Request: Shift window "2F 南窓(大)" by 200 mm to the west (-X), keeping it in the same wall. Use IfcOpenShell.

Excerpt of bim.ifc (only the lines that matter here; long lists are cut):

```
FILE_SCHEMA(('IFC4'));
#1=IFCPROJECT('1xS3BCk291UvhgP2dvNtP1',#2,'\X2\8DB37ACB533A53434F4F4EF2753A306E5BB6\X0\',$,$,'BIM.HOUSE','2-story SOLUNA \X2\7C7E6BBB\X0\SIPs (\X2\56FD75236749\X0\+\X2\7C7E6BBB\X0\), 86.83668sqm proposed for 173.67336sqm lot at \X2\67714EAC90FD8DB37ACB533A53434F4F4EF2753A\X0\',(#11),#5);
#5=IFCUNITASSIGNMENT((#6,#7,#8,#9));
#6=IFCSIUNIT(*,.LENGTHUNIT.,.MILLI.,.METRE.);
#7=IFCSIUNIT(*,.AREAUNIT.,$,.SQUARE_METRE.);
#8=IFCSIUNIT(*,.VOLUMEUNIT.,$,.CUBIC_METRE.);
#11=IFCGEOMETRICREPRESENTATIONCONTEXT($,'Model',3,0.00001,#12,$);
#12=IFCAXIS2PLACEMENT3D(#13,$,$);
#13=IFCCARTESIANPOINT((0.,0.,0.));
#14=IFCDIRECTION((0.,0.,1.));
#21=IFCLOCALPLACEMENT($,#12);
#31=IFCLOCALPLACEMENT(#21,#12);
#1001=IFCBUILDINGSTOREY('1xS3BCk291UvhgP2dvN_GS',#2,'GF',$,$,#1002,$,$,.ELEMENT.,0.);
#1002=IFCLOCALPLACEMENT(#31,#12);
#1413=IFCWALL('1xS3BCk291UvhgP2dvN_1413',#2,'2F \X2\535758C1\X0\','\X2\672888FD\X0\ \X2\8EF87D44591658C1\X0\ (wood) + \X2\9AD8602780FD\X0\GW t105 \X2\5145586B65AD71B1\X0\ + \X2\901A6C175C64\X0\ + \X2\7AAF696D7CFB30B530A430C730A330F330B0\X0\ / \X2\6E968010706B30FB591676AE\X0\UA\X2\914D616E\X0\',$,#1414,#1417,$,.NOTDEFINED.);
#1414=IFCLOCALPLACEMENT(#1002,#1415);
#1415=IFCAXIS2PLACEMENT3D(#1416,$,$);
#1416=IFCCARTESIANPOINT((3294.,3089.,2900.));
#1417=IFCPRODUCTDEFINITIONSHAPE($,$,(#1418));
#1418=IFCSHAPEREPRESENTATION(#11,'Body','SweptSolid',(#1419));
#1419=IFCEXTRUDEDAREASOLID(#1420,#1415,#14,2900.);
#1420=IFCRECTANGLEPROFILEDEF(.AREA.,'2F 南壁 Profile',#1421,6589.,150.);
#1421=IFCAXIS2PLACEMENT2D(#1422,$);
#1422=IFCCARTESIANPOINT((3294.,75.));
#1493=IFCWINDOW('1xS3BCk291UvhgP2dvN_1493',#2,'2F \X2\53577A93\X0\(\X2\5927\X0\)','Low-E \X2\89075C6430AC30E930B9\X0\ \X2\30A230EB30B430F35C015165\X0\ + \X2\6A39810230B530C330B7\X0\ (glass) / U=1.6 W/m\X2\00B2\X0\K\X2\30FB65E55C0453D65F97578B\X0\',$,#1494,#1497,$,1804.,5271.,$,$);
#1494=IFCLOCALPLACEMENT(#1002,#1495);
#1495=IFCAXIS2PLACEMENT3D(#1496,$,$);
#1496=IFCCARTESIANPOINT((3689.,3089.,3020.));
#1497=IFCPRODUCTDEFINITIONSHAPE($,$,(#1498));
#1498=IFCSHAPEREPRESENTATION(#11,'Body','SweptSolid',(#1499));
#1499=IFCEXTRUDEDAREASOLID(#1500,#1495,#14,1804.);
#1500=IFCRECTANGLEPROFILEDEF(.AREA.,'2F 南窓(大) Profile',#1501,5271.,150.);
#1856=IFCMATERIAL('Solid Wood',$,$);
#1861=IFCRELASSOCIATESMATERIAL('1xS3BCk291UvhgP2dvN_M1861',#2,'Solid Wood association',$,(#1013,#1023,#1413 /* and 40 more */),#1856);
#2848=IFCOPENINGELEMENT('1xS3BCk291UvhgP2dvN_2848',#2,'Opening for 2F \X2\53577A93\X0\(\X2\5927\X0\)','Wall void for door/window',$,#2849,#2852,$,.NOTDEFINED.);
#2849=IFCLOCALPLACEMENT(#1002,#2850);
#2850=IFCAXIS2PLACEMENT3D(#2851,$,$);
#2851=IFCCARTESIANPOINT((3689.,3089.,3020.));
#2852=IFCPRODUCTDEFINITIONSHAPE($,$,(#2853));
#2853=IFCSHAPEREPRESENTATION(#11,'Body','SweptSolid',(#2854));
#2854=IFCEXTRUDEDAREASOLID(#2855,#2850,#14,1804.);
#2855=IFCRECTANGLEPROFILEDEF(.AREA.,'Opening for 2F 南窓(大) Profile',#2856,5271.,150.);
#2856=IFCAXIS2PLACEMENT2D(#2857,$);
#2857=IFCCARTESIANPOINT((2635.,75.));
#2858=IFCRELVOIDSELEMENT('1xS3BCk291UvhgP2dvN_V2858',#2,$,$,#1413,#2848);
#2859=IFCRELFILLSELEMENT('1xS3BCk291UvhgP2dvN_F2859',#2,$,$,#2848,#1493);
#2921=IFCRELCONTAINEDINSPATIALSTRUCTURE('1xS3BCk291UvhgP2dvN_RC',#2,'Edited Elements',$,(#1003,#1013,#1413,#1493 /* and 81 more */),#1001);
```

```python
import ifcopenshell
import ifcopenshell.api.geometry
import ifcopenshell.util.placement
import ifcopenshell.util.unit

model = ifcopenshell.open("bim.ifc")
unit_scale = ifcopenshell.util.unit.calculate_unit_scale(model)

window = model.by_guid("1xS3BCk291UvhgP2dvN_1493")
opening = window.FillsVoids[0].RelatingOpeningElement
wall = opening.VoidsElements[0].RelatingBuildingElement

wall_matrix = ifcopenshell.util.placement.get_local_placement(wall.ObjectPlacement)
shift = wall_matrix[:3, 0] * -0.2 / unit_scale
before = ifcopenshell.util.placement.get_local_placement(window.ObjectPlacement)[:3, 3].copy()

# The window is not placed relative to its opening, so move both.
for product in (opening, window):
    matrix = ifcopenshell.util.placement.get_local_placement(product.ObjectPlacement)
    matrix[:3, 3] += shift
    ifcopenshell.api.geometry.edit_object_placement(model, product=product, matrix=matrix, is_si=False)

after = ifcopenshell.util.placement.get_local_placement(window.ObjectPlacement)[:3, 3]
print("window moved by", (after - before).round(3) + 0.0)

model.write("bim_v2.ifc")
```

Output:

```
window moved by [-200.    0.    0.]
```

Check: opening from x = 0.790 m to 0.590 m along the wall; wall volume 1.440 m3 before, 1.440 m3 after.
